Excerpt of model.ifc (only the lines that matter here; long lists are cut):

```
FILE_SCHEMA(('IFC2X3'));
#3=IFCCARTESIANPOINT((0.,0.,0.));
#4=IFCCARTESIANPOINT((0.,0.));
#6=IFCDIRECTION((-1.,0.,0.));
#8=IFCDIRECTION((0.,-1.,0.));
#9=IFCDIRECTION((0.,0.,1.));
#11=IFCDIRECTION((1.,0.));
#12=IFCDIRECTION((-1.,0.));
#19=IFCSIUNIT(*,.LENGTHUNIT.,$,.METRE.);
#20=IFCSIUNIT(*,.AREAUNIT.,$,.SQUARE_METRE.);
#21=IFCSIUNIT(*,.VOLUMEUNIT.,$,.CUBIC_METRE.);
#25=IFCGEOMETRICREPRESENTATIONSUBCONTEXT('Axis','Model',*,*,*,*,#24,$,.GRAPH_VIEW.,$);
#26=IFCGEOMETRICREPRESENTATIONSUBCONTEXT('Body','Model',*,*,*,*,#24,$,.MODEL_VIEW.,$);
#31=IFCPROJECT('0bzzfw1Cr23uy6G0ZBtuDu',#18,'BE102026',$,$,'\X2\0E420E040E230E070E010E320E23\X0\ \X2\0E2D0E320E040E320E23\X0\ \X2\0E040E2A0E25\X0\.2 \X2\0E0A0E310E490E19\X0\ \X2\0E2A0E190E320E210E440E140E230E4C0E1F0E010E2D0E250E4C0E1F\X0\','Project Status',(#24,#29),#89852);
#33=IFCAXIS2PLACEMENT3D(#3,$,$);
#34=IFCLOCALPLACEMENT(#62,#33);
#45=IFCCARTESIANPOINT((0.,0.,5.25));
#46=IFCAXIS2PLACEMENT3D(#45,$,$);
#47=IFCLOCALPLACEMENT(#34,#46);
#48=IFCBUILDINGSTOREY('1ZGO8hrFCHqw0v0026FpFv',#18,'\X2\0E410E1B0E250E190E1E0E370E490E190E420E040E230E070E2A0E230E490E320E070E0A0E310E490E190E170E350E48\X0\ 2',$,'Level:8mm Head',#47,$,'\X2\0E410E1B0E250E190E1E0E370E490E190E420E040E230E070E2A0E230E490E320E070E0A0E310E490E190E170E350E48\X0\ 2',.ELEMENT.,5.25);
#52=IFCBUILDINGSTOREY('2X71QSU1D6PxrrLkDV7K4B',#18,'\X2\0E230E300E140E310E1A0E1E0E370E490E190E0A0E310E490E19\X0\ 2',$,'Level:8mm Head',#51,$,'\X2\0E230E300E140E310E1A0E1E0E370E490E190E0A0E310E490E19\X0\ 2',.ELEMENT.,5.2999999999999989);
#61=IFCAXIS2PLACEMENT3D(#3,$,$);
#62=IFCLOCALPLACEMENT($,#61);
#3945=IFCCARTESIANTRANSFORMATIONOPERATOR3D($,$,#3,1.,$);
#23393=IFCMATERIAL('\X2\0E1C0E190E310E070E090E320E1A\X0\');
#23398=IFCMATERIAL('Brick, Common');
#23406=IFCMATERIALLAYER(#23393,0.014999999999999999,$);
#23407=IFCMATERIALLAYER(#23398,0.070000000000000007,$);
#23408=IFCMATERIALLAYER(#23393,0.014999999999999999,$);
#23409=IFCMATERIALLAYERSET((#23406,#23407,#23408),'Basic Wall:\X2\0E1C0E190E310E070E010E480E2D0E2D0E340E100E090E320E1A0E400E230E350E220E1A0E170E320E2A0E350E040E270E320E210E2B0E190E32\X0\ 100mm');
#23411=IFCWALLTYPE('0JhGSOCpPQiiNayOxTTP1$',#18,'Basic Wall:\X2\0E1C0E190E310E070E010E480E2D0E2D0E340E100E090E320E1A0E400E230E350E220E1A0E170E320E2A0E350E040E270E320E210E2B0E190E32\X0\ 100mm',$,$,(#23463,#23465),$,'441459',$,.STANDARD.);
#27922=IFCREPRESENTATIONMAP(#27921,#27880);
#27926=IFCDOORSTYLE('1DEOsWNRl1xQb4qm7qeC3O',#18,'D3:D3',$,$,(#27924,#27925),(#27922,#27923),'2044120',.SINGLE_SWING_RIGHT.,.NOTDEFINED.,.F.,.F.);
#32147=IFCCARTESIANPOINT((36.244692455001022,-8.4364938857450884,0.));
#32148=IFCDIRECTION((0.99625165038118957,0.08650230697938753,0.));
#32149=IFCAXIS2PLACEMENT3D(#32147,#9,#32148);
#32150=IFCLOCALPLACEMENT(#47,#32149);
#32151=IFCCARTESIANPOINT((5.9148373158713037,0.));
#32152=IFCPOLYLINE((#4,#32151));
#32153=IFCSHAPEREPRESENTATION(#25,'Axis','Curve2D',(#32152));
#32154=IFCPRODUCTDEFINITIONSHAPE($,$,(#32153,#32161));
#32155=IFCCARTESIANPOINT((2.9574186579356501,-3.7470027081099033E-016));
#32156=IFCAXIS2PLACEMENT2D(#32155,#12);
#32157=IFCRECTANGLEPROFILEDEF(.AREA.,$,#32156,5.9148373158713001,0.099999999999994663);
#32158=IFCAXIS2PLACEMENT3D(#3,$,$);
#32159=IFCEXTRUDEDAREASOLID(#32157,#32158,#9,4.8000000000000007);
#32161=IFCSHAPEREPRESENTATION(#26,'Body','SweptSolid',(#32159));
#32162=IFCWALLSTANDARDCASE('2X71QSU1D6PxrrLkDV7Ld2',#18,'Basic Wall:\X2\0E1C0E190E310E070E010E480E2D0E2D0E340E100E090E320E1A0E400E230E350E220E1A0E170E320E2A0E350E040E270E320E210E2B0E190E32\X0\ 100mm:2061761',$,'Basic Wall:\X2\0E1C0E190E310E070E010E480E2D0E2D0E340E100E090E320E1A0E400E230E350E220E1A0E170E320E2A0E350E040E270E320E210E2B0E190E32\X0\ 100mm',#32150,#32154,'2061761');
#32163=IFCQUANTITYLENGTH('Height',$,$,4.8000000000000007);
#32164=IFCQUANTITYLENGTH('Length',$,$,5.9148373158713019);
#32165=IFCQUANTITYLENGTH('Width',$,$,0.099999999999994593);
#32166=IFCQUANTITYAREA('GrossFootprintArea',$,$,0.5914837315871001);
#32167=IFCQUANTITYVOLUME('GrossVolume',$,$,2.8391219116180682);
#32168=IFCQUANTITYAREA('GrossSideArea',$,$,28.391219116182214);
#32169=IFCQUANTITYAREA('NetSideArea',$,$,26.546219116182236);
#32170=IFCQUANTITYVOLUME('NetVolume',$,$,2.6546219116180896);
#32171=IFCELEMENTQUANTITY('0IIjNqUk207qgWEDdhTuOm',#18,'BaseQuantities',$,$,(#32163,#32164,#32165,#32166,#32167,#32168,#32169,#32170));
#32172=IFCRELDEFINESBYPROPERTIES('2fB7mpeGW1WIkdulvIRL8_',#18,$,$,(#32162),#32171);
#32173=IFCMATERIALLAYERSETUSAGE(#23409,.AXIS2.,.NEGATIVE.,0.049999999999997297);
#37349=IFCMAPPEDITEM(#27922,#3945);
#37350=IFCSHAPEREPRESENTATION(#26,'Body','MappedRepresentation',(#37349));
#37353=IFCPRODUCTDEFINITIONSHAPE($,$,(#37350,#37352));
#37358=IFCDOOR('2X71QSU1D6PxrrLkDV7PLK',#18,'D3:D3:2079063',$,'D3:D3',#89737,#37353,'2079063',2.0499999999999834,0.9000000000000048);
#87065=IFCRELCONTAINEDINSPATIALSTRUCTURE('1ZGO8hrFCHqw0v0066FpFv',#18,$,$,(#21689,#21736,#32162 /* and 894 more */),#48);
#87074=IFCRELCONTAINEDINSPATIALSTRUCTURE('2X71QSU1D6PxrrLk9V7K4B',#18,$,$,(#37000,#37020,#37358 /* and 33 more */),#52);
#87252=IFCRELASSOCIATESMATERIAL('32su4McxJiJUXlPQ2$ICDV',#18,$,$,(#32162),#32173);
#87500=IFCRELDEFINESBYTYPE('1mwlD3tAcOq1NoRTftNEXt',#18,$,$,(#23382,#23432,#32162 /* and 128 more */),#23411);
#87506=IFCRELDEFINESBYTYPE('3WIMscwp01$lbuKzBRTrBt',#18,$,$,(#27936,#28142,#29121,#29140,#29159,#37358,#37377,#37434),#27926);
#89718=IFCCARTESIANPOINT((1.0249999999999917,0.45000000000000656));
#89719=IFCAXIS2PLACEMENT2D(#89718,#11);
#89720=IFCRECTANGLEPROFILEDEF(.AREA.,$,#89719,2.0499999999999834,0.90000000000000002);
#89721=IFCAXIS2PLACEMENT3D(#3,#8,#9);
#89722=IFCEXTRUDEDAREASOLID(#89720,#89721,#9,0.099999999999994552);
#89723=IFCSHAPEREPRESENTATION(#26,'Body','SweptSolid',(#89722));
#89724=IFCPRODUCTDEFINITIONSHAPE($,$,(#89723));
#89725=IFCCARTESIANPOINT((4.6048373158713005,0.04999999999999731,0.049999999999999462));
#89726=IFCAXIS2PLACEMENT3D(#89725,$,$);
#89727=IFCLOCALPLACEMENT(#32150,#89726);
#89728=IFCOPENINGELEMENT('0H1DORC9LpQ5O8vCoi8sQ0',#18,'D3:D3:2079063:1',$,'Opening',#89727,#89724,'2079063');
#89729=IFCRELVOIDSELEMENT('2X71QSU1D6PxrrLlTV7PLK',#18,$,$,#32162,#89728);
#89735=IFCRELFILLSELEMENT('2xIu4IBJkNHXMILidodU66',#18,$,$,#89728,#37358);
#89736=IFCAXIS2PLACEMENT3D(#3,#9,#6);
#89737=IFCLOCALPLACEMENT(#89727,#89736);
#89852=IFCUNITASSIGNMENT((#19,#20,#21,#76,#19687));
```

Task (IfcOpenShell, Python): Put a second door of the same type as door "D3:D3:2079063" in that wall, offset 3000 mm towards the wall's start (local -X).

```python
import ifcopenshell
import ifcopenshell.api.feature
import ifcopenshell.api.geometry
import ifcopenshell.api.pset
import ifcopenshell.api.root
import ifcopenshell.geom
import ifcopenshell.util.element
import ifcopenshell.util.placement
import ifcopenshell.util.shape
import ifcopenshell.util.unit

model = ifcopenshell.open("model.ifc")
area_scale = ifcopenshell.util.unit.calculate_unit_scale(model, "AREAUNIT")
volume_scale = ifcopenshell.util.unit.calculate_unit_scale(model, "VOLUMEUNIT")
settings = ifcopenshell.geom.settings()


def volume(element):
    """Net volume in cubic metres, openings subtracted."""
    shape = ifcopenshell.geom.create_shape(settings, element)
    return ifcopenshell.util.shape.get_volume(shape.geometry)


def reuse_history(source, copy):
    """copy_class also copies each property set's owner history, people and application; keep the originals."""
    for rel in copy.IsDefinedBy:
        if rel.is_a("IfcRelDefinesByProperties") and (history := rel.RelatingPropertyDefinition.OwnerHistory):
            rel.RelatingPropertyDefinition.OwnerHistory = source.OwnerHistory
            ifcopenshell.util.element.remove_deep2(model, history)


door = model.by_guid("2X71QSU1D6PxrrLkDV7PLK")
opening = door.FillsVoids[0].RelatingOpeningElement
wall = opening.VoidsElements[0].RelatingBuildingElement
before = volume(wall)
shift = ifcopenshell.util.placement.get_local_placement(wall.ObjectPlacement)[:3, 0] * -3.0

# copy_class copies the void relationship, type, container and properties, but no geometry.
new_opening = ifcopenshell.api.root.copy_class(model, product=opening)
new_opening.Representation = ifcopenshell.util.element.copy_deep(
    model, opening.Representation, exclude=["IfcGeometricRepresentationContext", "IfcRepresentationMap"]
)
new_opening.Name = "D3:D3"
new_opening.Tag = None
reuse_history(opening, new_opening)
new_door = ifcopenshell.api.root.copy_class(model, product=door)
new_door.Representation = ifcopenshell.util.element.copy_deep(
    model, door.Representation, exclude=["IfcGeometricRepresentationContext", "IfcRepresentationMap"]
)
new_door.Name = "D3:D3"
new_door.Tag = None
reuse_history(door, new_door)
fills = ifcopenshell.api.feature.add_filling(model, opening=new_opening, element=new_door)
fills.OwnerHistory = new_door.OwnerHistory  # required in IFC2X3

for old, new in ((opening, new_opening), (door, new_door)):
    matrix = ifcopenshell.util.placement.get_local_placement(old.ObjectPlacement)
    matrix[:3, 3] += shift
    ifcopenshell.api.geometry.edit_object_placement(model, product=new, matrix=matrix, is_si=False)

after = volume(wall)
thickness = 0.1  # wall thickness in metres

# Update the wall's stored quantities.
qto = model.by_id(ifcopenshell.util.element.get_pset(wall, "BaseQuantities", should_inherit=False)["id"])
ifcopenshell.api.pset.edit_qto(model, qto=qto, properties={
    "NetSideArea": after / thickness / area_scale,
    "NetVolume": after / volume_scale,
})

print(f"wall volume {before:.3f} -> {after:.3f} m3")

model.write("model_edited.ifc")
```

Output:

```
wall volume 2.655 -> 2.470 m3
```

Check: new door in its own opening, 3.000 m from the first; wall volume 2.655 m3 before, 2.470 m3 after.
